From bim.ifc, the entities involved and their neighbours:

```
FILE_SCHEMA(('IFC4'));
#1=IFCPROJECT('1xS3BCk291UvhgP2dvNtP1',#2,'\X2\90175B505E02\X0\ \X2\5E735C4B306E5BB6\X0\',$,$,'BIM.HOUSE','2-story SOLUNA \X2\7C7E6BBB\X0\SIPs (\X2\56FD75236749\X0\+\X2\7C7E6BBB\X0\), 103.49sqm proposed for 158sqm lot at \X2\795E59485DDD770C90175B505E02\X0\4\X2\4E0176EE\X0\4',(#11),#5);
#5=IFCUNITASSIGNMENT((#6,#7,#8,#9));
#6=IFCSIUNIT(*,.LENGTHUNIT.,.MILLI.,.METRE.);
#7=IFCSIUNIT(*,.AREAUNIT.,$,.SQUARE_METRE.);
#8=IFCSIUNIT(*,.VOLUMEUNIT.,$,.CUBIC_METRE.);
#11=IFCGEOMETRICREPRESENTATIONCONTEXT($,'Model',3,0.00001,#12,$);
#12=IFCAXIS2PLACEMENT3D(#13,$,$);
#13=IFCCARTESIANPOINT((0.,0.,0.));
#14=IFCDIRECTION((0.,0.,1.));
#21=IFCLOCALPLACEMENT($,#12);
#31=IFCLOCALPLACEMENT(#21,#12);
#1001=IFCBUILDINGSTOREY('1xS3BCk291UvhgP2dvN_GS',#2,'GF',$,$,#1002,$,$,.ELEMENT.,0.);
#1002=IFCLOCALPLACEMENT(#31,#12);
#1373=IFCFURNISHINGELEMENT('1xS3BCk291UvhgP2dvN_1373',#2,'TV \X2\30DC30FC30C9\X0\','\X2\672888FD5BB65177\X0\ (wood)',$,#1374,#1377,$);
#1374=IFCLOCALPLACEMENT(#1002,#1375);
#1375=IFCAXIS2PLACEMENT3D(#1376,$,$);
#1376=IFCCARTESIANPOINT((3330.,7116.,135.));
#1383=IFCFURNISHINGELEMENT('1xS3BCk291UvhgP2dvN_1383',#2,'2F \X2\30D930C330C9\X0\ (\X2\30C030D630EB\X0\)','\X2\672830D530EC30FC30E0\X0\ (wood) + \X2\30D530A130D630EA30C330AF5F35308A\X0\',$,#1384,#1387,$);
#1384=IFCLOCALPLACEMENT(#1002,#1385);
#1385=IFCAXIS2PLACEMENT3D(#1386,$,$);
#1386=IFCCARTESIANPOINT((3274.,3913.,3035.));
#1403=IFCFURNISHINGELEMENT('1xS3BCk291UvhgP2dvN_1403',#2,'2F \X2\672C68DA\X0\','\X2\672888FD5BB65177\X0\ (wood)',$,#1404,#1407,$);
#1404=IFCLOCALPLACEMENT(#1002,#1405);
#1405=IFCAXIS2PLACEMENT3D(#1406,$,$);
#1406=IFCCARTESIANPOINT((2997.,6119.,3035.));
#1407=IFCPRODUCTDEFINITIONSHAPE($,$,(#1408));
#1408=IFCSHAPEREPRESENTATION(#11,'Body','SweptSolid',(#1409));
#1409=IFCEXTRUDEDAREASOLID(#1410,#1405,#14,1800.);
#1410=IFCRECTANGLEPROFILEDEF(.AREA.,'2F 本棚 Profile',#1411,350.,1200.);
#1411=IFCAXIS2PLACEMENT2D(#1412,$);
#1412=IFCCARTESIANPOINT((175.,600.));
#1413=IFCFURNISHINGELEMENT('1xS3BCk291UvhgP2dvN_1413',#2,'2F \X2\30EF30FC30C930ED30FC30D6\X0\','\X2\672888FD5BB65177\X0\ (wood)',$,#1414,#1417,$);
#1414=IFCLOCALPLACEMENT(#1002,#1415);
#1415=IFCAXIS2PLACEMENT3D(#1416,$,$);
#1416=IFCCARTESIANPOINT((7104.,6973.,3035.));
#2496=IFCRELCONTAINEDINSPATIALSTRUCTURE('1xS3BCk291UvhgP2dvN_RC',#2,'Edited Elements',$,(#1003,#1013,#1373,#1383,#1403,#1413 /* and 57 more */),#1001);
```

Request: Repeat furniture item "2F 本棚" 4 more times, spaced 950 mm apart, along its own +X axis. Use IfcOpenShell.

```python
import ifcopenshell
import ifcopenshell.api.geometry
import ifcopenshell.api.root
import ifcopenshell.util.element
import ifcopenshell.util.placement

model = ifcopenshell.open("bim.ifc")


def reuse_history(source, copy):
    """copy_class also copies each property set's owner history, people and application; keep the originals."""
    for rel in copy.IsDefinedBy:
        if rel.is_a("IfcRelDefinesByProperties") and (history := rel.RelatingPropertyDefinition.OwnerHistory):
            rel.RelatingPropertyDefinition.OwnerHistory = source.OwnerHistory
            ifcopenshell.util.element.remove_deep2(model, history)


source = model.by_guid("1xS3BCk291UvhgP2dvN_1403")
base = ifcopenshell.util.placement.get_local_placement(source.ObjectPlacement)
step = base[:3, 0] * 950.0

for i in range(1, 5):
    copy = ifcopenshell.api.root.copy_class(model, product=source)
    copy.Representation = ifcopenshell.util.element.copy_deep(
        model, source.Representation, exclude=["IfcGeometricRepresentationContext", "IfcRepresentationMap"]
    )
    reuse_history(source, copy)
    matrix = base.copy()
    matrix[:3, 3] += i * step
    print("added at", matrix[:3, 3].round(3) + 0.0)
    ifcopenshell.api.geometry.edit_object_placement(model, product=copy, matrix=matrix, is_si=False)

model.write("bim-out.ifc")
```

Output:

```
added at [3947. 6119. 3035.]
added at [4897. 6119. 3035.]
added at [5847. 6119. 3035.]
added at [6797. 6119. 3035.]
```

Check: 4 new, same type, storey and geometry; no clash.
